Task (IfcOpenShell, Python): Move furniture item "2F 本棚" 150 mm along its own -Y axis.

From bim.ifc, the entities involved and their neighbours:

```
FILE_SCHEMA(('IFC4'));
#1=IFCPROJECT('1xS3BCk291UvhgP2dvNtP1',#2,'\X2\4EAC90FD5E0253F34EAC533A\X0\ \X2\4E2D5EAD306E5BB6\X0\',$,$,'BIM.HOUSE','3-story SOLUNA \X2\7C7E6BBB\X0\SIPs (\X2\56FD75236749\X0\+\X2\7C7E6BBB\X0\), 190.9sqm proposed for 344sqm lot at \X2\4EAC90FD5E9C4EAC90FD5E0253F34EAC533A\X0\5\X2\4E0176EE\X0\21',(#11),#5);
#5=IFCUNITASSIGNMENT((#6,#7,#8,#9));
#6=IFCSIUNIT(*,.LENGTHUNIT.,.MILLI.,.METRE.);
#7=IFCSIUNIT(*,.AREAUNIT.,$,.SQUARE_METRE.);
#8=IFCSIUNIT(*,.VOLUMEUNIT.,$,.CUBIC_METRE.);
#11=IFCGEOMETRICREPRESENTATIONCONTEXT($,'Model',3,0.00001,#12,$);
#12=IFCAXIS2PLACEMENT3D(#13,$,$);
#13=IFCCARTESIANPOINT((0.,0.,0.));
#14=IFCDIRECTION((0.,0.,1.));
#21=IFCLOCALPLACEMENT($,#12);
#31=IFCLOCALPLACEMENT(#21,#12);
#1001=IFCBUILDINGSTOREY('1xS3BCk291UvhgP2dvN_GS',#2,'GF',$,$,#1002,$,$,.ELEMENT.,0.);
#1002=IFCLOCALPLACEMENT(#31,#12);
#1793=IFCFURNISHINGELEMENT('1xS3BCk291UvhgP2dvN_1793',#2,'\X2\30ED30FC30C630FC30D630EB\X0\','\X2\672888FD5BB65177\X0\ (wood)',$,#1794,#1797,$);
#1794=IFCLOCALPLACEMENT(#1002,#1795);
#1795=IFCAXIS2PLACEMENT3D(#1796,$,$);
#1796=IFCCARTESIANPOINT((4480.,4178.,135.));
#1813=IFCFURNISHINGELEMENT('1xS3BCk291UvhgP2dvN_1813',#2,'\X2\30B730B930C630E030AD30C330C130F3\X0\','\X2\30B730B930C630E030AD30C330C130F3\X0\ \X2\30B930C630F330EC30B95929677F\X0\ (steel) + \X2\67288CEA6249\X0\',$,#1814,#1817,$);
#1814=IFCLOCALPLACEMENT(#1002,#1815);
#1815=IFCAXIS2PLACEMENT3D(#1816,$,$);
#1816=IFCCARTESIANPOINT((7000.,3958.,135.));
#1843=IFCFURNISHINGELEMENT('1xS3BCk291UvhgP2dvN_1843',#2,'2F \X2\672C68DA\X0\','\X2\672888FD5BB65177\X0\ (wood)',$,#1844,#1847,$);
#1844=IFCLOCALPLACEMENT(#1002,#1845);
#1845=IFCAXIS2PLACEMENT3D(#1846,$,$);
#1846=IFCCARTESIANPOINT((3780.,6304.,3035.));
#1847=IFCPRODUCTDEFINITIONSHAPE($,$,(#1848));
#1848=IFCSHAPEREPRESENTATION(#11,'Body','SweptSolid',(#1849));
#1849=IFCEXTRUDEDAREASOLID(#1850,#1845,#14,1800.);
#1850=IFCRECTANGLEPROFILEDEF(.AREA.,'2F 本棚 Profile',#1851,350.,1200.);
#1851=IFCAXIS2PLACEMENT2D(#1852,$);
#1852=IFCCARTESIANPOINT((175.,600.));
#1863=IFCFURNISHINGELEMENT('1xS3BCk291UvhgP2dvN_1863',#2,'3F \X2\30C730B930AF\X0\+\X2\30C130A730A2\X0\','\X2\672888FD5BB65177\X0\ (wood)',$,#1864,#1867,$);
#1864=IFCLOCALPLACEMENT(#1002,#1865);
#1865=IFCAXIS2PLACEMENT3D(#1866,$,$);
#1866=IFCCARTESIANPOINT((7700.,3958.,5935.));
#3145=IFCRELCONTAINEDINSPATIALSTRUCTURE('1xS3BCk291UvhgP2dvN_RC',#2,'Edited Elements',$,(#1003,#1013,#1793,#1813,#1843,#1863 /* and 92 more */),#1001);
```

```python
import ifcopenshell
import ifcopenshell.api.geometry
import ifcopenshell.util.placement
import ifcopenshell.util.unit

model = ifcopenshell.open("bim.ifc")
unit_scale = ifcopenshell.util.unit.calculate_unit_scale(model)

item = model.by_guid("1xS3BCk291UvhgP2dvN_1843")
matrix = ifcopenshell.util.placement.get_local_placement(item.ObjectPlacement)
matrix[:3, 3] -= matrix[:3, 1] * 0.15 / unit_scale
ifcopenshell.api.geometry.edit_object_placement(model, product=item, matrix=matrix, is_si=False)

print(ifcopenshell.util.placement.get_local_placement(item.ObjectPlacement).round(3) + 0.0)

model.write("bim_v2.ifc")
```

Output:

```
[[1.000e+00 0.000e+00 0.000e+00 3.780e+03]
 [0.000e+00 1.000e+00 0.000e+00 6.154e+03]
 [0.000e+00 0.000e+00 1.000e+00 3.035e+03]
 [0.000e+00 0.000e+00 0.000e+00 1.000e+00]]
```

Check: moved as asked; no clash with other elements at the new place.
